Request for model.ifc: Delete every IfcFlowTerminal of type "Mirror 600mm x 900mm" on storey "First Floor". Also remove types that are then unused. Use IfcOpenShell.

First a look at what the model holds.

```python
import ifcopenshell
import ifcopenshell.util.element

model = ifcopenshell.open("model.ifc")
print(model.schema)
storey = next(s for s in model.by_type("IfcBuildingStorey") if s.Name == "First Floor")
terminals = [e for e in ifcopenshell.util.element.get_decomposition(storey) if e.is_a("IfcFlowTerminal")]
seen = {}
for e in terminals:
    element_type = ifcopenshell.util.element.get_type(e)
    name = element_type.Name if element_type not in (None, e) else None
    seen[name] = seen.get(name, 0) + 1
for name, count in sorted(seen.items(), key=str):
    print(count, "x", name)
```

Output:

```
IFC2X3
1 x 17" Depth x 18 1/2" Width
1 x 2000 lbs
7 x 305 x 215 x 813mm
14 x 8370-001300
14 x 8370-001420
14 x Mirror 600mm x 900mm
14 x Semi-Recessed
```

```python
import ifcopenshell
import ifcopenshell.api.root
import ifcopenshell.util.element

model = ifcopenshell.open("model.ifc")

storey = next(s for s in model.by_type("IfcBuildingStorey") if s.Name == "First Floor")
terminals = [e for e in ifcopenshell.util.element.get_decomposition(storey) if e.is_a("IfcFlowTerminal")]
targets = [e for e in terminals if (t := ifcopenshell.util.element.get_type(e)) not in (None, e) and t.Name == "Mirror 600mm x 900mm"]
types = {ifcopenshell.util.element.get_type(e) for e in targets} - {None, *targets}

for e in targets:
    ifcopenshell.api.root.remove_product(model, product=e)
print(len(targets), "removed")

unused = [t for t in types if not ifcopenshell.util.element.get_types(t)]
for t in unused:
    ifcopenshell.api.root.remove_product(model, product=t)
print(len(unused), "unused types removed")

model.write("model-out.ifc")
```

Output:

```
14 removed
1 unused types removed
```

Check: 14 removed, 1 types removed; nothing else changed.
